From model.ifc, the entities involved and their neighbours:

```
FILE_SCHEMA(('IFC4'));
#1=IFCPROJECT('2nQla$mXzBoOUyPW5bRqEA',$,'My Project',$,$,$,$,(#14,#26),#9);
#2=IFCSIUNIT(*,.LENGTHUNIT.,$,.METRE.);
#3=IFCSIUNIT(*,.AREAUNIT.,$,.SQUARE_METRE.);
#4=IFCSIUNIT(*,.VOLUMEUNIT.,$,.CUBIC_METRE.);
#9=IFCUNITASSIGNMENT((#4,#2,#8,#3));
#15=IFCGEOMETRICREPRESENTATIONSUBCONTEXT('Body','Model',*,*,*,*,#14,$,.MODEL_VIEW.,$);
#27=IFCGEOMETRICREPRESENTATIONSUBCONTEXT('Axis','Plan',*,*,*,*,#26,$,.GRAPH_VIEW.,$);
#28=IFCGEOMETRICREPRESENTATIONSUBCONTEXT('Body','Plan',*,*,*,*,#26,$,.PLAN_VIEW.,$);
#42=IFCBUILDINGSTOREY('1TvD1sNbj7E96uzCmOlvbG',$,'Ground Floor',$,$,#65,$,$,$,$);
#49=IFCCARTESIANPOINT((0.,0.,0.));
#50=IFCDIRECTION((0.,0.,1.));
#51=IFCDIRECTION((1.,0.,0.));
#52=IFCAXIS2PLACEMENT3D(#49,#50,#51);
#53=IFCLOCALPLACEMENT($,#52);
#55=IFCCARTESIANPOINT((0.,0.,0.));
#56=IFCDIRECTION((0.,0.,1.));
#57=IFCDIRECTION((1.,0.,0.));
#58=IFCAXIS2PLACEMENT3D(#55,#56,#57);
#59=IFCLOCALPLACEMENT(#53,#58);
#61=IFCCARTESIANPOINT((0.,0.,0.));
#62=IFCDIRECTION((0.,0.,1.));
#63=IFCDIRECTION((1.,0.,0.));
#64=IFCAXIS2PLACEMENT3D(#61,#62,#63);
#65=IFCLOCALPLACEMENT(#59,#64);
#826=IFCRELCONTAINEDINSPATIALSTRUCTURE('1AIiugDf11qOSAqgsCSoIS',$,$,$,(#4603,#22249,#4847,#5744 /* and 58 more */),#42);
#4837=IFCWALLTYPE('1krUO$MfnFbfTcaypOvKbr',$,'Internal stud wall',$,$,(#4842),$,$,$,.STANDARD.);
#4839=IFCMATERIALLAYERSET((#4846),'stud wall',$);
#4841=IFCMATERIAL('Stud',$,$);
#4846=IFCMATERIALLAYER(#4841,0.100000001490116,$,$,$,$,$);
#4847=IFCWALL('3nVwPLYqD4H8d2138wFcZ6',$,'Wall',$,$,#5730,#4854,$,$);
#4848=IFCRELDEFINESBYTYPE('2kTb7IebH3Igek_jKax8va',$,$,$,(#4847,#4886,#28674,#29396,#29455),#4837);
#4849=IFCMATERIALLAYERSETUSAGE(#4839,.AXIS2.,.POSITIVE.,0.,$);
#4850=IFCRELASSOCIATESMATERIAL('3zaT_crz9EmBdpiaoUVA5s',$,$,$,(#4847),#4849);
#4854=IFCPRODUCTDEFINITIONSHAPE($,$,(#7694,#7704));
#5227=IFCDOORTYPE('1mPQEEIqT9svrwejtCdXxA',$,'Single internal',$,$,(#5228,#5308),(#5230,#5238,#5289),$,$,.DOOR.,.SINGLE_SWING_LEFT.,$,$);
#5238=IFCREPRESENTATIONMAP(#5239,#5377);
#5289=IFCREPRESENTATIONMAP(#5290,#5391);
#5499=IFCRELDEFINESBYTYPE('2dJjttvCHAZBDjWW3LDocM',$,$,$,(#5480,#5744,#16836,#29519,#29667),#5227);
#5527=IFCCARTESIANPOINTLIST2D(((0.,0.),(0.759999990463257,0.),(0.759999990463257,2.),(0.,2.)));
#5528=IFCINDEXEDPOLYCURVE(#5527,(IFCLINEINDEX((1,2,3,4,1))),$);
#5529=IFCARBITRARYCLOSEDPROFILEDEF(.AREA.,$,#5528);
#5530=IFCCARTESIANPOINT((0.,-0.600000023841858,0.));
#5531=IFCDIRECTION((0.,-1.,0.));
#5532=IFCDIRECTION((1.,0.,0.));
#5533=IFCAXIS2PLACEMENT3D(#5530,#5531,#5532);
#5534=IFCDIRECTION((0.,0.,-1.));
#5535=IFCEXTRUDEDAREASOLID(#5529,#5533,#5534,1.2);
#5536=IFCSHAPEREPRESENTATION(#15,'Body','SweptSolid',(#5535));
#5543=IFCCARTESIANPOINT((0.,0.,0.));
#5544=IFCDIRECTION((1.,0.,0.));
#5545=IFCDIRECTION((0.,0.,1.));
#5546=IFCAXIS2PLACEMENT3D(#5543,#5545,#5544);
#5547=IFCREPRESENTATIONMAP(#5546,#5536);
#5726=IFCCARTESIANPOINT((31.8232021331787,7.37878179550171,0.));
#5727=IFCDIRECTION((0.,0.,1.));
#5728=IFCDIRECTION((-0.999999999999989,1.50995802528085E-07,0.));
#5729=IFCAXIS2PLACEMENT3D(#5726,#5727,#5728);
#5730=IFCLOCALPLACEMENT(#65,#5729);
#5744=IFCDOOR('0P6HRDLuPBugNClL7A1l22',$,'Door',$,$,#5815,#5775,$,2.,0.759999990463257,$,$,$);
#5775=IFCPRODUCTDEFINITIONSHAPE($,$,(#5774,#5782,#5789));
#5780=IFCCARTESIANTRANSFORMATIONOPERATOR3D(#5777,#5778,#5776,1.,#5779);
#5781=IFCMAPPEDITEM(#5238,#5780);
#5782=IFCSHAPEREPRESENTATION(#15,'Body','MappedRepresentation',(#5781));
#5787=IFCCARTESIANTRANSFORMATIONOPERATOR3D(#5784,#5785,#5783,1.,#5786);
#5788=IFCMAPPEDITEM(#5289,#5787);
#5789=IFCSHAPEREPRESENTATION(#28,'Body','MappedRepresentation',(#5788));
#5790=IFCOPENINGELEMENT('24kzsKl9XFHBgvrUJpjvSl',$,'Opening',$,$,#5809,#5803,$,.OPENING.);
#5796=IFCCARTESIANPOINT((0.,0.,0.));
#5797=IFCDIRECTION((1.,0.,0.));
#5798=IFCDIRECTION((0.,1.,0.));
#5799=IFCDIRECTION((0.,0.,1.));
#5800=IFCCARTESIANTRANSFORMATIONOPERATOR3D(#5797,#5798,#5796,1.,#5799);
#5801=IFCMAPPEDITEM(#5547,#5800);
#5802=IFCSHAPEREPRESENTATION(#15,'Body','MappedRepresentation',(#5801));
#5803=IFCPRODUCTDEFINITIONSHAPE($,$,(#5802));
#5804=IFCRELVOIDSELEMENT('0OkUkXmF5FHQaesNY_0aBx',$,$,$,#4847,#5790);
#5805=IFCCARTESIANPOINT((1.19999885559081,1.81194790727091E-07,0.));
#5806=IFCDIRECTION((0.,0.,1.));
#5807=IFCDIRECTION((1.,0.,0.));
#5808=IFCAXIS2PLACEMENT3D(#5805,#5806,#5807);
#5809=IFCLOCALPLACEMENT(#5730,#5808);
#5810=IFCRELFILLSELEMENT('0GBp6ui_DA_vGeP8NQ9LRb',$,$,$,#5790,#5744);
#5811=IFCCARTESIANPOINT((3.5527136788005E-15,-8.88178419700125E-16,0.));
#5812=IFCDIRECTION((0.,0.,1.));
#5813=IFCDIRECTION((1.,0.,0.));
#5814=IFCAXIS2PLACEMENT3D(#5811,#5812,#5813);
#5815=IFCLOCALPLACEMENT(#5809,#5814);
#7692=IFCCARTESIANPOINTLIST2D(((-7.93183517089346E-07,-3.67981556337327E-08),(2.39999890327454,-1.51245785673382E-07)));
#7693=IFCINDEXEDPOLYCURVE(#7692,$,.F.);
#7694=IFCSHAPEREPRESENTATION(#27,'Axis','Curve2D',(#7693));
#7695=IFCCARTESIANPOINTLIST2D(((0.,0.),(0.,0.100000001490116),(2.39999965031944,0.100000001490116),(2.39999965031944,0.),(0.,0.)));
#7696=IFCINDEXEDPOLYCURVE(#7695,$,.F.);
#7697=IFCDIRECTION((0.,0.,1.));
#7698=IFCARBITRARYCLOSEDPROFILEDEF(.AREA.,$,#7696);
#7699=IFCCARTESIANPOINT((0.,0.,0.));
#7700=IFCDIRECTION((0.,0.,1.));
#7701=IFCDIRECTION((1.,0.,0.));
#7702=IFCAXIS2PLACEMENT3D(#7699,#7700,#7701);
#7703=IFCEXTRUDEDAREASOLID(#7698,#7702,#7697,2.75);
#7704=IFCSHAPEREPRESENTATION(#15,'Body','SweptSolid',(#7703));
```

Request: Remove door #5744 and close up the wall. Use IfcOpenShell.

```python
import ifcopenshell
import ifcopenshell.api.feature
import ifcopenshell.api.root
import ifcopenshell.geom
import ifcopenshell.util.shape

model = ifcopenshell.open("model.ifc")
settings = ifcopenshell.geom.settings()


def volume(element):
    """Net volume in cubic metres, openings subtracted."""
    shape = ifcopenshell.geom.create_shape(settings, element)
    return ifcopenshell.util.shape.get_volume(shape.geometry)


door = model.by_id(5744)
opening = door.FillsVoids[0].RelatingOpeningElement
wall = opening.VoidsElements[0].RelatingBuildingElement
before = volume(wall)

ifcopenshell.api.root.remove_product(model, product=door)
ifcopenshell.api.feature.remove_feature(model, feature=opening)

after = volume(wall)

print(f"wall volume {before:.3f} -> {after:.3f} m3")

model.write("model_rev.ifc")
```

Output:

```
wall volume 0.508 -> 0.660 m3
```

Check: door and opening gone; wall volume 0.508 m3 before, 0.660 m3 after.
